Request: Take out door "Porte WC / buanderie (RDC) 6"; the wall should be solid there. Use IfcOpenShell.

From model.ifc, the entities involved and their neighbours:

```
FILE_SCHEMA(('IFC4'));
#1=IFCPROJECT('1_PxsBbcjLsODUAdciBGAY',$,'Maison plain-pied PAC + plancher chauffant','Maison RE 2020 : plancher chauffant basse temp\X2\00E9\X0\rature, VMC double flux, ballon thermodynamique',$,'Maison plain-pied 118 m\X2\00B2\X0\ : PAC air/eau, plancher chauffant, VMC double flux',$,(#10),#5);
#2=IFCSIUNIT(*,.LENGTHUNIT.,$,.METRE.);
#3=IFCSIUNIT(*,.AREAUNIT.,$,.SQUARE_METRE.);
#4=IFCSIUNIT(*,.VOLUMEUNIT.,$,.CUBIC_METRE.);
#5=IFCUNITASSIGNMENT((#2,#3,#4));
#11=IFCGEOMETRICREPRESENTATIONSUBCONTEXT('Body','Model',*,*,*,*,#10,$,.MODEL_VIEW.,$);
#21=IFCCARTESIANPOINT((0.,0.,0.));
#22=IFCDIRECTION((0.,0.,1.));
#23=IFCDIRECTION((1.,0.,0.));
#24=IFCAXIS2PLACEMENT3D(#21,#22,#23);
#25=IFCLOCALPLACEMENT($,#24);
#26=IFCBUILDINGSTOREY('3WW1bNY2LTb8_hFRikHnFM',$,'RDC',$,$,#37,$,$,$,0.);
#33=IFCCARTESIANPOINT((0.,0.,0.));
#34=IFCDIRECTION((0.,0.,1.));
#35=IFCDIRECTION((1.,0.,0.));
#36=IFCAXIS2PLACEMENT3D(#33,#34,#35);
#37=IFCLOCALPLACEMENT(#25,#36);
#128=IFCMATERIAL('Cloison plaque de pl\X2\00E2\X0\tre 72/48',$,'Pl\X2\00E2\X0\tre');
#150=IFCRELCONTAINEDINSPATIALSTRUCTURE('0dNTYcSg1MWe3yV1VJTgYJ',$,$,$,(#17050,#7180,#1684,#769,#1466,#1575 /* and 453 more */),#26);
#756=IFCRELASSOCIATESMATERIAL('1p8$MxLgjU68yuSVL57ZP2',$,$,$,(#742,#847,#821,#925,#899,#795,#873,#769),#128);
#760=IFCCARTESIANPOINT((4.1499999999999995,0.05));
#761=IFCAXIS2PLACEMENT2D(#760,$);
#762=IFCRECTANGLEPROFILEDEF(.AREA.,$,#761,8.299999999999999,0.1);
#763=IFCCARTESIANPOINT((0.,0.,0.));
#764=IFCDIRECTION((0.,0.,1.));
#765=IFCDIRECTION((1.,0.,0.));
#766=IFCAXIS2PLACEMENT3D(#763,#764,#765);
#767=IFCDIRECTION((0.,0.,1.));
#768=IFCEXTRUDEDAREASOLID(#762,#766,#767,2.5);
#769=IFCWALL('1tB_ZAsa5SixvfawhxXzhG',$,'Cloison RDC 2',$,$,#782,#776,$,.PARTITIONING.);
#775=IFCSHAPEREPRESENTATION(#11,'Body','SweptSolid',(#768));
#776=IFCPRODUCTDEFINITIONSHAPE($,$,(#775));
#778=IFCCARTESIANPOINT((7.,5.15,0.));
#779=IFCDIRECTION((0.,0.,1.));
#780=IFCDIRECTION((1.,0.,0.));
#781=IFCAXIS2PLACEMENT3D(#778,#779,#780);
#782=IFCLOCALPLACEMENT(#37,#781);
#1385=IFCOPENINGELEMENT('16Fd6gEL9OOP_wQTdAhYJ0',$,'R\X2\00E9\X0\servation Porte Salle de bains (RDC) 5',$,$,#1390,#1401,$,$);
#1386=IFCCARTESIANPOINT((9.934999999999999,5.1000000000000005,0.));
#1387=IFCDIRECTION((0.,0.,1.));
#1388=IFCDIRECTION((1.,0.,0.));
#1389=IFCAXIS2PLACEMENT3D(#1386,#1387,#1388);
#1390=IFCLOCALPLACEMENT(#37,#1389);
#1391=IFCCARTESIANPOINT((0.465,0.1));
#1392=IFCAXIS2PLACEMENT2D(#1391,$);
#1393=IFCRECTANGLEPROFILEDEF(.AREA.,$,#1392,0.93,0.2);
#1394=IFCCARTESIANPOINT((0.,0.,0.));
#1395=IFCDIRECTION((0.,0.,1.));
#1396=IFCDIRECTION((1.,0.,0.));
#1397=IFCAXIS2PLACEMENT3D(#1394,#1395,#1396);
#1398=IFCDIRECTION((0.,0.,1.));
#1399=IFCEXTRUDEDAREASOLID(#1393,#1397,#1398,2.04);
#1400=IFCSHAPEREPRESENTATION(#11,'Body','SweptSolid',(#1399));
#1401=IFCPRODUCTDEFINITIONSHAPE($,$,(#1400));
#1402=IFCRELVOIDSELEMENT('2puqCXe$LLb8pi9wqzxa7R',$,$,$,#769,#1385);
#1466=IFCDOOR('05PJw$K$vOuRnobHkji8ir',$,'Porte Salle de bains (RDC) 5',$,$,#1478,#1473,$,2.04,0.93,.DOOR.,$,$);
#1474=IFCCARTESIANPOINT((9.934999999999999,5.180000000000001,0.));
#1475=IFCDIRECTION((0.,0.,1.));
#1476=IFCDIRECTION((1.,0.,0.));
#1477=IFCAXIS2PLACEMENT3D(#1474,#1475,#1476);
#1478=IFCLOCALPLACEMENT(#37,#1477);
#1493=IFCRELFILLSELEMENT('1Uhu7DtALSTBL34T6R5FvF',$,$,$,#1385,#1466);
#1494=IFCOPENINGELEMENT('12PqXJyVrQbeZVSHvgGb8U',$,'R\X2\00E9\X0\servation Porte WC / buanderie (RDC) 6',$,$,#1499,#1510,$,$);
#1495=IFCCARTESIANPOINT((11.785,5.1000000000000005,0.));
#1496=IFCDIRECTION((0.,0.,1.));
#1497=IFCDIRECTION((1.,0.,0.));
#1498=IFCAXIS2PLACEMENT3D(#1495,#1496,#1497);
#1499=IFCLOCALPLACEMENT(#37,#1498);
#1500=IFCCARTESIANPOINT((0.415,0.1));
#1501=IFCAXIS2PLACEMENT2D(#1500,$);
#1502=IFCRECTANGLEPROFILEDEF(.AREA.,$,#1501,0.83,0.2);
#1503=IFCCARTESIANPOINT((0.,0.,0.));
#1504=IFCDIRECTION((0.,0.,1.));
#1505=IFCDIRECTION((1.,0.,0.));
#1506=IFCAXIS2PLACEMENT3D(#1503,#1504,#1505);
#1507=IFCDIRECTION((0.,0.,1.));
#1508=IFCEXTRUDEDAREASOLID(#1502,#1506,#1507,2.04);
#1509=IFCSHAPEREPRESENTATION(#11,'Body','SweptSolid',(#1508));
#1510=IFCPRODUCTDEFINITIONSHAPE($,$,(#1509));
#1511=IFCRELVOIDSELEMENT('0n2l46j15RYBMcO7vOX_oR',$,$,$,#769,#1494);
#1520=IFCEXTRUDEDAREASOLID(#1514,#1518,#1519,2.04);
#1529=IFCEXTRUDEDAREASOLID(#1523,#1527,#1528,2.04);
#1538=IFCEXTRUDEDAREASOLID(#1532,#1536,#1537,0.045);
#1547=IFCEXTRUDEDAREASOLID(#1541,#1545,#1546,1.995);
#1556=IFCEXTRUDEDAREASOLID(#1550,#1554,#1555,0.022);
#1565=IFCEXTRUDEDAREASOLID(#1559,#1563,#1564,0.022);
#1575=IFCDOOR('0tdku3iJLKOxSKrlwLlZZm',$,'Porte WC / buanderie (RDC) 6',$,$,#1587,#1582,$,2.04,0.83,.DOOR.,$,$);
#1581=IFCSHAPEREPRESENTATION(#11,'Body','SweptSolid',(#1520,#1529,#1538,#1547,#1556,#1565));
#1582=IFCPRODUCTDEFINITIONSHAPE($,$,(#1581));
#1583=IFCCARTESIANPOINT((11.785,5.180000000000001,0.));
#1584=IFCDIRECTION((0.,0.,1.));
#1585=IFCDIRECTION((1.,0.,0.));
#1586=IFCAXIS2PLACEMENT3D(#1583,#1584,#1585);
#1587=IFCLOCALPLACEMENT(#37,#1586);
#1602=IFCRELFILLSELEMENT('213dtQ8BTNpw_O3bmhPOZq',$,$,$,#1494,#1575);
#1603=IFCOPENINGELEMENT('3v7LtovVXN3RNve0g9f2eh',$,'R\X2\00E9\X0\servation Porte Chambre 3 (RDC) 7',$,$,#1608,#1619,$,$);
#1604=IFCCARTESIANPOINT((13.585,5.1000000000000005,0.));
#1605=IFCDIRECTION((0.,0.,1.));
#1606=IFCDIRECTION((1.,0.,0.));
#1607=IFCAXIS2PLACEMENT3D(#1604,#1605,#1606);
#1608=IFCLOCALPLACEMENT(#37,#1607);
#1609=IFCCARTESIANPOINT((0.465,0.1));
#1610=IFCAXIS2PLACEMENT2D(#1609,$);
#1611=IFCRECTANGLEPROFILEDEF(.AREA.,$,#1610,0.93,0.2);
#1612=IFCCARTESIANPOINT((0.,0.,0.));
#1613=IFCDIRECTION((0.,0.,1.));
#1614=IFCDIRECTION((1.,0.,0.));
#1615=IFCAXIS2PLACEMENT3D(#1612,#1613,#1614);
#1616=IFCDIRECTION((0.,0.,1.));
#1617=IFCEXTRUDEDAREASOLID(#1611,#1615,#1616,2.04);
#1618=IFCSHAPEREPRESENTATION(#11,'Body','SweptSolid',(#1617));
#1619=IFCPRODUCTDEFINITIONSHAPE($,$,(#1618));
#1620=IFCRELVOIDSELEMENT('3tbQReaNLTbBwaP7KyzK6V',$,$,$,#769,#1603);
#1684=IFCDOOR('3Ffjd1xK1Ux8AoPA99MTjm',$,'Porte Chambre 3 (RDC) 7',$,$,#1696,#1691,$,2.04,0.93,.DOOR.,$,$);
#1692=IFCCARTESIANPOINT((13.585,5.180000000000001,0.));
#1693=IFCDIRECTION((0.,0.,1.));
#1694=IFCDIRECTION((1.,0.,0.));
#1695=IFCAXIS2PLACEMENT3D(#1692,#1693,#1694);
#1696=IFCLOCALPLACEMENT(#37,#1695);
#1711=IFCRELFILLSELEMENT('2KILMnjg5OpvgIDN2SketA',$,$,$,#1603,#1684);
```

```python
import ifcopenshell
import ifcopenshell.api.feature
import ifcopenshell.api.root
import ifcopenshell.geom
import ifcopenshell.util.shape

model = ifcopenshell.open("model.ifc")
settings = ifcopenshell.geom.settings()


def volume(element):
    """Net volume in cubic metres, openings subtracted."""
    shape = ifcopenshell.geom.create_shape(settings, element)
    return ifcopenshell.util.shape.get_volume(shape.geometry)


door = model.by_id(1575)
opening = door.FillsVoids[0].RelatingOpeningElement
wall = opening.VoidsElements[0].RelatingBuildingElement
before = volume(wall)

ifcopenshell.api.root.remove_product(model, product=door)
ifcopenshell.api.feature.remove_feature(model, feature=opening)

after = volume(wall)

print(f"wall volume {before:.3f} -> {after:.3f} m3")

model.write("model_updated.ifc")
```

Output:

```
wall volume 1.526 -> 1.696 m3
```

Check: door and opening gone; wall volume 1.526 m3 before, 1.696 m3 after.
